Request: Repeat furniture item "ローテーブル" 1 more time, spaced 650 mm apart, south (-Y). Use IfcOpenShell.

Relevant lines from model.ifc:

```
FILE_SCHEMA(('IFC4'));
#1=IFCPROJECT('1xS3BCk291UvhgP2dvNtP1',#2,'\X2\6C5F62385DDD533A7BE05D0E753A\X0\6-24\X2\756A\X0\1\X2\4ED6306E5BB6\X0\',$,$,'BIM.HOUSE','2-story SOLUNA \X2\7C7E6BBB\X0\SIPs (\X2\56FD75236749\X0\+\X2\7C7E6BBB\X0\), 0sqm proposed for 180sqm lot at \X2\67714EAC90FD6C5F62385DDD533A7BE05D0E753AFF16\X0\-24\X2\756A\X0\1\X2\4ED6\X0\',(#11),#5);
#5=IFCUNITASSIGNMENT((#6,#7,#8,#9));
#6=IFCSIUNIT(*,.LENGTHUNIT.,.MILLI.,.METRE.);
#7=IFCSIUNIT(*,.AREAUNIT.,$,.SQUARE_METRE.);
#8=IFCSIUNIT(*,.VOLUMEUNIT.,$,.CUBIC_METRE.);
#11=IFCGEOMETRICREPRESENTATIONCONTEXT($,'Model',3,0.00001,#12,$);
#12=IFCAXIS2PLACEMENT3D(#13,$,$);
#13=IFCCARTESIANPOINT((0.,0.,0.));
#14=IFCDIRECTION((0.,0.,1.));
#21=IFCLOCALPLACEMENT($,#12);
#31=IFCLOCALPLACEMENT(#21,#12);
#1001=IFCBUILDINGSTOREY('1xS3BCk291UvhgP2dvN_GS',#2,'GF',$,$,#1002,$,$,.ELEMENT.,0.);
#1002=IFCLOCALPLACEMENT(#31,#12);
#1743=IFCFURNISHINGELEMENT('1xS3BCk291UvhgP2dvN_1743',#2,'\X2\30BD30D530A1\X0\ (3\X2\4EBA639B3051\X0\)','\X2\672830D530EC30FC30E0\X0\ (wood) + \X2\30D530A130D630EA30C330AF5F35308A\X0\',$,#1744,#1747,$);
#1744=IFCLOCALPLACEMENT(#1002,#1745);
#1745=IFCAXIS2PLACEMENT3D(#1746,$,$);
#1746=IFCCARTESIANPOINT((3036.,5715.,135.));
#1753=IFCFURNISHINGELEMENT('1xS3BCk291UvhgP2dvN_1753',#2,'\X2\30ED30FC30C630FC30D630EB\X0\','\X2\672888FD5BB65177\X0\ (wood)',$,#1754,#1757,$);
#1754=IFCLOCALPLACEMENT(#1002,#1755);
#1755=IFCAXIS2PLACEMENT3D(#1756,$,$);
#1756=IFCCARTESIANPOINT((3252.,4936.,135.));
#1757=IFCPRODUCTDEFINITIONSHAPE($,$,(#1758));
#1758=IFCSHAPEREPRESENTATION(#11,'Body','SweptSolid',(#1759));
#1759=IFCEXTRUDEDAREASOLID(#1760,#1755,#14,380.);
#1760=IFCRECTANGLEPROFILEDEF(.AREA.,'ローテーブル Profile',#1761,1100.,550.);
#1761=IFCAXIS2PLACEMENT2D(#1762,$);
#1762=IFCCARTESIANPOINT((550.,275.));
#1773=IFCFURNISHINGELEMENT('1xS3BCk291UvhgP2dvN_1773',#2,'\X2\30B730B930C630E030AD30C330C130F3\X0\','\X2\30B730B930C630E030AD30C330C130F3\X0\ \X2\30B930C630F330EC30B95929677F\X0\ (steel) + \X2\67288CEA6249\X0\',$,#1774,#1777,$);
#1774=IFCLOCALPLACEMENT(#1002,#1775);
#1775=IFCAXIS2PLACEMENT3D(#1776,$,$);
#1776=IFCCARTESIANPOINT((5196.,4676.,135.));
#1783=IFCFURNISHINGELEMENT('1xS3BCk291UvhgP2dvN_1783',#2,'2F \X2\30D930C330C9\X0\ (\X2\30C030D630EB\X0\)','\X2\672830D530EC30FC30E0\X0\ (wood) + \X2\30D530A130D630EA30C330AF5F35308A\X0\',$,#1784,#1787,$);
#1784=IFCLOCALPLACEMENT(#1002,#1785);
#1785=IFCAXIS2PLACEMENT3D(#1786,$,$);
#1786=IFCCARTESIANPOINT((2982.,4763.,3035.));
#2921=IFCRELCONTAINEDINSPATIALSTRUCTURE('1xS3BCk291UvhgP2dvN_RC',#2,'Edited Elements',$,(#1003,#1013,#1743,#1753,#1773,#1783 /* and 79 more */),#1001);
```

```python
import numpy as np
import ifcopenshell
import ifcopenshell.api.geometry
import ifcopenshell.api.root
import ifcopenshell.util.element
import ifcopenshell.util.placement
import ifcopenshell.util.unit

model = ifcopenshell.open("model.ifc")
unit_scale = ifcopenshell.util.unit.calculate_unit_scale(model)


def reuse_history(source, copy):
    """copy_class also copies each property set's owner history, people and application; keep the originals."""
    for rel in copy.IsDefinedBy:
        if rel.is_a("IfcRelDefinesByProperties") and (history := rel.RelatingPropertyDefinition.OwnerHistory):
            rel.RelatingPropertyDefinition.OwnerHistory = source.OwnerHistory
            ifcopenshell.util.element.remove_deep2(model, history)


source = model.by_guid("1xS3BCk291UvhgP2dvN_1753")
base = ifcopenshell.util.placement.get_local_placement(source.ObjectPlacement)
step = np.array([0.0, -1.0, 0.0]) * 0.65 / unit_scale

for i in range(1, 2):
    copy = ifcopenshell.api.root.copy_class(model, product=source)
    copy.Representation = ifcopenshell.util.element.copy_deep(
        model, source.Representation, exclude=["IfcGeometricRepresentationContext", "IfcRepresentationMap"]
    )
    reuse_history(source, copy)
    matrix = base.copy()
    matrix[:3, 3] += i * step
    print("added at", matrix[:3, 3].round(3) + 0.0)
    ifcopenshell.api.geometry.edit_object_placement(model, product=copy, matrix=matrix, is_si=False)

model.write("model_rev.ifc")
```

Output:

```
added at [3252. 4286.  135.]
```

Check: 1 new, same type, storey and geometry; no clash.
